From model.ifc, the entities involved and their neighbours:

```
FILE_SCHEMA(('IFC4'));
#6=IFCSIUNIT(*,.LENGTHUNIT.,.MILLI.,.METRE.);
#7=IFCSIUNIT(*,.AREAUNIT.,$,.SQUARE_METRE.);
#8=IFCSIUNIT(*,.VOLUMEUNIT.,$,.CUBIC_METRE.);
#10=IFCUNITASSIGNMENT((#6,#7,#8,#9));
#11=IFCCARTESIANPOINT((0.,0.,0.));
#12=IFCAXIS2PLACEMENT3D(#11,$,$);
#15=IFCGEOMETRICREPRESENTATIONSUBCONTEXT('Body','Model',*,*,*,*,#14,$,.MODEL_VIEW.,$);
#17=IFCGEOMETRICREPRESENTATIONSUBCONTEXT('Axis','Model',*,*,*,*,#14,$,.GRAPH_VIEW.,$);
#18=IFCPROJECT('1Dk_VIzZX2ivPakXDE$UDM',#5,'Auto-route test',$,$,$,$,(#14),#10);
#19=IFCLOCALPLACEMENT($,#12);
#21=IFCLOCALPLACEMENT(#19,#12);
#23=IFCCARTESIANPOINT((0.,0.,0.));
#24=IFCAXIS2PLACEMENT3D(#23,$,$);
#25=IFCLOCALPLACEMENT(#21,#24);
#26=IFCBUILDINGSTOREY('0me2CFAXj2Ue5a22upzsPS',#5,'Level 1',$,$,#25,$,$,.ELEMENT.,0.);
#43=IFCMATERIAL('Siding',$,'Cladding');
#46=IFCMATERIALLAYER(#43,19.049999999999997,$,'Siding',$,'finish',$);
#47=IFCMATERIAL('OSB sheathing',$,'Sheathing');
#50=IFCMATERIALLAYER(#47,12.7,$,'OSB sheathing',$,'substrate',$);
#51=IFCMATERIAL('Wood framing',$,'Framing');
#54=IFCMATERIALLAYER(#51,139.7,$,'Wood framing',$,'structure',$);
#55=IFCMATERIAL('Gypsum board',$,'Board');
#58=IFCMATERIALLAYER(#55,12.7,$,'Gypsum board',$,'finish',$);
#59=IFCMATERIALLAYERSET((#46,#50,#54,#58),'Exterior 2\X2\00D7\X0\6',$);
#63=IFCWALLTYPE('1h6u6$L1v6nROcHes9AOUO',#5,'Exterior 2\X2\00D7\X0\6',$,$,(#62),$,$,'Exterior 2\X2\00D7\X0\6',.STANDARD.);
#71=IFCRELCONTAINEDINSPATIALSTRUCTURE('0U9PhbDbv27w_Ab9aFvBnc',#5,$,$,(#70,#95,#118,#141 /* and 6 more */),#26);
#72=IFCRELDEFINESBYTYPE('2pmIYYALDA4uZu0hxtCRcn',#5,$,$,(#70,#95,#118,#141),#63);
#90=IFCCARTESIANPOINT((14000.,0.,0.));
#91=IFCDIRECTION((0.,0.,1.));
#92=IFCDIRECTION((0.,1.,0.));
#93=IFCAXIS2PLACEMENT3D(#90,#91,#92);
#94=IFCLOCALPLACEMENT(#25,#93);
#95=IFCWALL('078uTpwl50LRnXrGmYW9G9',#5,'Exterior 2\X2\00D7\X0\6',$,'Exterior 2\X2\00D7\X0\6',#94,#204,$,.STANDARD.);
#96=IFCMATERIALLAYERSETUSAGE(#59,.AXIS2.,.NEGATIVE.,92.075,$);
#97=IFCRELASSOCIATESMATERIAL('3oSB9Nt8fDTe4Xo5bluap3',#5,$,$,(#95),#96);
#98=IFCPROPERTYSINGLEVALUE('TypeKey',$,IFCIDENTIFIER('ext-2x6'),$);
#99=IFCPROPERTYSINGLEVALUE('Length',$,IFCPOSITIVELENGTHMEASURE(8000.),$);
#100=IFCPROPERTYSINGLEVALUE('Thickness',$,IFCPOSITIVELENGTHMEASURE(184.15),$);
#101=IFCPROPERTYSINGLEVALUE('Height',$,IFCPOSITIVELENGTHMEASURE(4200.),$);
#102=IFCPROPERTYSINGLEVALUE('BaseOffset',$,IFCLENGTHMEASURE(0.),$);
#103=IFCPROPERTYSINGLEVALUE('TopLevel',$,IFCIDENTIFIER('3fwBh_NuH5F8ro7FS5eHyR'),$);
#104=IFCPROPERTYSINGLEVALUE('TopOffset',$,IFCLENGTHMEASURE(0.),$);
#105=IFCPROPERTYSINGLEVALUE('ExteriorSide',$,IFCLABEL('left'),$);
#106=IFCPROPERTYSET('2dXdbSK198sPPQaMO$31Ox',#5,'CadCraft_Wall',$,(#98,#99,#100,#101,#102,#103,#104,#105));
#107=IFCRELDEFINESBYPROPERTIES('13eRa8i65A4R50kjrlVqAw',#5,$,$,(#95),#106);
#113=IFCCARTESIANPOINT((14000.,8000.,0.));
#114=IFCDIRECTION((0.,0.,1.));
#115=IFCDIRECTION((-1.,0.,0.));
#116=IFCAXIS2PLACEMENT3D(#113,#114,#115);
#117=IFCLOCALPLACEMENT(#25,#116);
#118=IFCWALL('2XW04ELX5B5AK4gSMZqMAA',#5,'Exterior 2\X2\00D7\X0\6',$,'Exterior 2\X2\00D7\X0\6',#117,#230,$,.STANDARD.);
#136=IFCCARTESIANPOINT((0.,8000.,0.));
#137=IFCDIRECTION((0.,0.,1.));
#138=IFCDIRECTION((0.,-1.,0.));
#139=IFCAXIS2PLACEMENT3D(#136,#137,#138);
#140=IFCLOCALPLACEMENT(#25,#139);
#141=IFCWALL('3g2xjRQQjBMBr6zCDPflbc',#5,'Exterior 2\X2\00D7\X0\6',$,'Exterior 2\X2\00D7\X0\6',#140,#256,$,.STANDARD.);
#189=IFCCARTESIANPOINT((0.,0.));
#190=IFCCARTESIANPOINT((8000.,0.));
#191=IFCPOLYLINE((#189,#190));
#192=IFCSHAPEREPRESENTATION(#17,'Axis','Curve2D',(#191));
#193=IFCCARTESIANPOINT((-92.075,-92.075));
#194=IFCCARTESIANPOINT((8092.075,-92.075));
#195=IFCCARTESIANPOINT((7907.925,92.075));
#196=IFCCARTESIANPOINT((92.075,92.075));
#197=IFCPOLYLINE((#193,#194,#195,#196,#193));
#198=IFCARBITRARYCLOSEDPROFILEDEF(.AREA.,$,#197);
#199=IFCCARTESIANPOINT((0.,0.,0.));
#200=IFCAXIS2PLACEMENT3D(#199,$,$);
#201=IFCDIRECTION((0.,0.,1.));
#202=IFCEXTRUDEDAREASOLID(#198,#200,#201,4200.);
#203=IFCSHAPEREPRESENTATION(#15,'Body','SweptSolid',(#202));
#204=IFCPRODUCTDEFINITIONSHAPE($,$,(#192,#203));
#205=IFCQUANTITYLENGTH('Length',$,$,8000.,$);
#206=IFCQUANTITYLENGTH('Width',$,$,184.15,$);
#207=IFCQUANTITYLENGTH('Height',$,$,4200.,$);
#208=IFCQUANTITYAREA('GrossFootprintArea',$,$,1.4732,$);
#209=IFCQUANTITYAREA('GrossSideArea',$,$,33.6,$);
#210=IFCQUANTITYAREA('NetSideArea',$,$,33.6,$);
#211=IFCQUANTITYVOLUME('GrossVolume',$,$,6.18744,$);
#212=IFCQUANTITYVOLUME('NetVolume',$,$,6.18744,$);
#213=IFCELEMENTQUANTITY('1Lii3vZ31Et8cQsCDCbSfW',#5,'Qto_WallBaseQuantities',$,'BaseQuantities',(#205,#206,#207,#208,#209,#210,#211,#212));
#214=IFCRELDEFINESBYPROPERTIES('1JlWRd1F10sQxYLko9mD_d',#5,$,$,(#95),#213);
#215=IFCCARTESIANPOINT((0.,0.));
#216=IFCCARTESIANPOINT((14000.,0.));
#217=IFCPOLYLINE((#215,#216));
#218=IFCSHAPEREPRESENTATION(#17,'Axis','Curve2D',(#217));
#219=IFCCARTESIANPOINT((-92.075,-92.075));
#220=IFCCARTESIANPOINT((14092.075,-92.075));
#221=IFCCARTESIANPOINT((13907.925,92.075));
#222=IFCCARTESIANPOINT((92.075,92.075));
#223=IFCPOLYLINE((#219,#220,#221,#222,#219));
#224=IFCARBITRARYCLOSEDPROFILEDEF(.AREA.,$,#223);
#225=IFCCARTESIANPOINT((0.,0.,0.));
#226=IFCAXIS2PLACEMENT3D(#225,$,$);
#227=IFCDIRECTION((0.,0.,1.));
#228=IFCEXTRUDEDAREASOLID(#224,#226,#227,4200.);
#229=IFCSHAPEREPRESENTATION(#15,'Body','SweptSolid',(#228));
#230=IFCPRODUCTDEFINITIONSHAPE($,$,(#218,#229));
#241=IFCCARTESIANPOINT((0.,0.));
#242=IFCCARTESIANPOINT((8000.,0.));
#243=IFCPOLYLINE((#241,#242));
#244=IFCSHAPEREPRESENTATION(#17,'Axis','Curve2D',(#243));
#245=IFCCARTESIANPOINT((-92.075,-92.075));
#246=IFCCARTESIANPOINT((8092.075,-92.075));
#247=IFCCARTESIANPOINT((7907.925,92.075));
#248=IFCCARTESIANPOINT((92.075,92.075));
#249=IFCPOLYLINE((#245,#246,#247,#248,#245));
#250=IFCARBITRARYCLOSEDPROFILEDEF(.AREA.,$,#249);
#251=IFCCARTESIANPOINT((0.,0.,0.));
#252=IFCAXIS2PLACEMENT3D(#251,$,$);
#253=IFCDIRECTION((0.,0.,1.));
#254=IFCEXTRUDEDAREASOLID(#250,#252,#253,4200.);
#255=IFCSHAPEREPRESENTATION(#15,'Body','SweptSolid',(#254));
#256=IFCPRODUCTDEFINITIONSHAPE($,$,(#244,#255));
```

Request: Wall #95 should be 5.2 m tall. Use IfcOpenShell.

```python
import ifcopenshell
import ifcopenshell.api.pset
import ifcopenshell.geom
import ifcopenshell.util.element
import ifcopenshell.util.representation
import ifcopenshell.util.shape
import ifcopenshell.util.unit

model = ifcopenshell.open("model.ifc")
unit_scale = ifcopenshell.util.unit.calculate_unit_scale(model)
area_scale = ifcopenshell.util.unit.calculate_unit_scale(model, "AREAUNIT")
volume_scale = ifcopenshell.util.unit.calculate_unit_scale(model, "VOLUMEUNIT")
settings = ifcopenshell.geom.settings()


def volume(element):
    """Net volume in cubic metres, openings subtracted."""
    shape = ifcopenshell.geom.create_shape(settings, element)
    return ifcopenshell.util.shape.get_volume(shape.geometry)


wall = model.by_guid("078uTpwl50LRnXrGmYW9G9")
before = volume(wall)

body = ifcopenshell.util.representation.get_representation(wall, "Model", "Body")
solid = body.Items[0]
old_height = solid.Depth
solid.Depth = 5.2 / unit_scale
after = volume(wall)
thickness = 0.1841  # wall thickness in metres

# Update the stored height, areas and volumes.
pset = model.by_id(ifcopenshell.util.element.get_pset(wall, "CadCraft_Wall", should_inherit=False)["id"])
ifcopenshell.api.pset.edit_pset(model, pset=pset, properties={
    "Height": model.create_entity("IfcPositiveLengthMeasure", solid.Depth),
})
qto = model.by_id(ifcopenshell.util.element.get_pset(wall, "Qto_WallBaseQuantities", should_inherit=False)["id"])
ifcopenshell.api.pset.edit_qto(model, qto=qto, properties={
    "Height": solid.Depth,
    "GrossSideArea": ifcopenshell.util.element.get_pset(wall, "Qto_WallBaseQuantities", "GrossSideArea") * solid.Depth / old_height,
    "NetSideArea": after / thickness / area_scale,
    "GrossVolume": ifcopenshell.util.element.get_pset(wall, "Qto_WallBaseQuantities", "GrossVolume") * solid.Depth / old_height,
    "NetVolume": after / volume_scale,
})

print(f"height {old_height:g} -> {solid.Depth:g}, volume {before:.3f} -> {after:.3f} m3")

model.write("model_v2.ifc")
```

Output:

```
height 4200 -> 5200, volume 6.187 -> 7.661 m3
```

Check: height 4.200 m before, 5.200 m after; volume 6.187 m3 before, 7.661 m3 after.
